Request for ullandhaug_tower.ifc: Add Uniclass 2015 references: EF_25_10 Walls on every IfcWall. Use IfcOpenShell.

First a look at what the model holds.

```python
import ifcopenshell

model = ifcopenshell.open("ullandhaug_tower.ifc")
print(model.schema)
print("classifications:", [c.Name for c in model.by_type("IfcClassification")])
for ifc_class in ("IfcDoor", "IfcRoof", "IfcStair", "IfcWall", "IfcWindow"):
    print(ifc_class, len(model.by_type(ifc_class)))
```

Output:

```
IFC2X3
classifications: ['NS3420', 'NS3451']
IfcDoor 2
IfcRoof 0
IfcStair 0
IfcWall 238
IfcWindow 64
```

```python
import ifcopenshell
import ifcopenshell.api.classification

model = ifcopenshell.open("ullandhaug_tower.ifc")

# IFC2X3 requires Source and Edition and has no link from the project to the system.
system = model.create_entity("IfcClassification", Source="NBS", Edition="2015", Name="Uniclass 2015")

codes = {
    "IfcWall": ("EF_25_10", "Walls"),
}
for ifc_class, (code, name) in codes.items():
    products = model.by_type(ifc_class)
    ifcopenshell.api.classification.add_reference(
        model, products=products, classification=system, identification=code, name=name
    )
    print(code, len(products))

model.write("ullandhaug_tower_rev.ifc")
```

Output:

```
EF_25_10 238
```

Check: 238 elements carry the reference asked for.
